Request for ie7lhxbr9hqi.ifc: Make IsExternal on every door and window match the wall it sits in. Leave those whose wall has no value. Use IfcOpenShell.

First a look at what the model holds.

```python
import ifcopenshell
import ifcopenshell.util.element

model = ifcopenshell.open("ie7lhxbr9hqi.ifc")
print(model.schema)
seen = {}
for e in model.by_type("IfcDoor") + model.by_type("IfcWindow"):
    if not e.FillsVoids:
        continue
    host = e.FillsVoids[0].RelatingOpeningElement.VoidsElements[0].RelatingBuildingElement
    own = ifcopenshell.util.element.get_pset(e, f"Pset_{e.is_a()[3:].removesuffix('StandardCase')}Common", "IsExternal")
    wall = ifcopenshell.util.element.get_pset(host, "Pset_WallCommon", "IsExternal")
    seen[e.is_a(), own, wall] = seen.get((e.is_a(), own, wall), 0) + 1
for (cls, own, wall), count in sorted(seen.items(), key=str):
    print(count, cls, "IsExternal:", own, "| host wall:", wall)
```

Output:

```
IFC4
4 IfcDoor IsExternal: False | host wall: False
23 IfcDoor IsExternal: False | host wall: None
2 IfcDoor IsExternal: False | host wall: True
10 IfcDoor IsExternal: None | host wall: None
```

```python
import ifcopenshell
import ifcopenshell.api.pset
import ifcopenshell.util.element

model = ifcopenshell.open("ie7lhxbr9hqi.ifc")

count = 0
for ifc_class, pset_name in (("IfcDoor", "Pset_DoorCommon"), ("IfcWindow", "Pset_WindowCommon")):
    for e in model.by_type(ifc_class):
        if not e.FillsVoids:
            continue
        host = e.FillsVoids[0].RelatingOpeningElement.VoidsElements[0].RelatingBuildingElement
        external = ifcopenshell.util.element.get_pset(host, "Pset_WallCommon", "IsExternal")
        if external is None or ifcopenshell.util.element.get_pset(e, pset_name, "IsExternal") == external:
            continue
        pset = ifcopenshell.api.pset.add_pset(model, product=e, name=pset_name)
        ifcopenshell.api.pset.edit_pset(model, pset=pset, properties={"IsExternal": external})
        count += 1

print(count, "updated")

model.write("ie7lhxbr9hqi_v2.ifc")
```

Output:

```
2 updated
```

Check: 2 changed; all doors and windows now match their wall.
